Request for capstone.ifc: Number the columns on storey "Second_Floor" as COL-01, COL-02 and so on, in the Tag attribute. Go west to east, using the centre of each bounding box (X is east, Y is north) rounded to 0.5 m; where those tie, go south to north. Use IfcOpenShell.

First a look at what the model holds.

```python
import ifcopenshell
import ifcopenshell.util.element
import ifcopenshell.util.placement

model = ifcopenshell.open("capstone.ifc")
print(model.schema)
storey = next(s for s in model.by_type("IfcBuildingStorey") if s.Name == "Second_Floor")
columns = [e for e in ifcopenshell.util.element.get_decomposition(storey) if e.is_a("IfcColumn")]
for e in sorted(columns, key=lambda e: e.id()):
    origin = ifcopenshell.util.placement.get_local_placement(e.ObjectPlacement)[:3, 3]
    print(e.id(), e.Tag, e.Name, origin.round(2) + 0.0, sep=" | ")
```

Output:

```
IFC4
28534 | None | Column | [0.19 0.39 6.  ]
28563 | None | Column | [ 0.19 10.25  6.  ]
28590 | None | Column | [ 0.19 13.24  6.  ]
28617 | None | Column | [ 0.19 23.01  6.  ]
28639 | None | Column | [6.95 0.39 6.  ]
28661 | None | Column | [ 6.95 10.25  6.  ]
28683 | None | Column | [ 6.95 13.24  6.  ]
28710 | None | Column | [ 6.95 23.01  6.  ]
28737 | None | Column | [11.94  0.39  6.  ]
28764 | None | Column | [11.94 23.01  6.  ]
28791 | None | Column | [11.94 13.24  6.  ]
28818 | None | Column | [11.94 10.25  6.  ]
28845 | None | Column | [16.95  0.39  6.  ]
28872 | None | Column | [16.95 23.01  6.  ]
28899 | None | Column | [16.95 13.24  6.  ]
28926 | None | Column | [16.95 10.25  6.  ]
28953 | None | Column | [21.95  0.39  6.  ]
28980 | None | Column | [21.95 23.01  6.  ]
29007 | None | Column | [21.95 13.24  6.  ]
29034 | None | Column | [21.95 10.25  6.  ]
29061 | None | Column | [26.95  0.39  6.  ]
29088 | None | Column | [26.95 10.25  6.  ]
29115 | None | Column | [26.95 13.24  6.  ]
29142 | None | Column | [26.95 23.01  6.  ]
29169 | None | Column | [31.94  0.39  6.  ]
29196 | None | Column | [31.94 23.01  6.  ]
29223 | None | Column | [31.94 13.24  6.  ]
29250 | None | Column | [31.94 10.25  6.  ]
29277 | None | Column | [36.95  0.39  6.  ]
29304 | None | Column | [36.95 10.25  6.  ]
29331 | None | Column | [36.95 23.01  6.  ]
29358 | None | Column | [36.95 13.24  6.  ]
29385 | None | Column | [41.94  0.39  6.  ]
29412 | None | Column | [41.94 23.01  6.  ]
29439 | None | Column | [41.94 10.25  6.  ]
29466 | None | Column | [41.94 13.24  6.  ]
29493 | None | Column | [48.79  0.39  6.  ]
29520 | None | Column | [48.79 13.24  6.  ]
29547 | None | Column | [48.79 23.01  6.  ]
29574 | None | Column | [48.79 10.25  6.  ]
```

```python
import ifcopenshell
import ifcopenshell.geom
import ifcopenshell.util.element
import ifcopenshell.util.shape

model = ifcopenshell.open("capstone.ifc")
settings = ifcopenshell.geom.settings()
settings.set("use-world-coords", True)


def centre(element):
    shape = ifcopenshell.geom.create_shape(settings, element)
    return ifcopenshell.util.shape.get_bbox_centroid(shape.geometry)


storey = next(s for s in model.by_type("IfcBuildingStorey") if s.Name == "Second_Floor")
columns = [e for e in ifcopenshell.util.element.get_decomposition(storey) if e.is_a("IfcColumn")]

# Insertion points can sit at a corner or the storey origin, so sort by the geometry (in metres).
centres = {e: centre(e) for e in columns}
columns.sort(key=lambda e: (round(centres[e][0] / 0.5), centres[e][1]))

for i, e in enumerate(columns, start=1):
    number = f"COL-{i:02d}"
    e.Tag = number
    print(e.id(), number)

model.write("capstone_rev.ifc")
```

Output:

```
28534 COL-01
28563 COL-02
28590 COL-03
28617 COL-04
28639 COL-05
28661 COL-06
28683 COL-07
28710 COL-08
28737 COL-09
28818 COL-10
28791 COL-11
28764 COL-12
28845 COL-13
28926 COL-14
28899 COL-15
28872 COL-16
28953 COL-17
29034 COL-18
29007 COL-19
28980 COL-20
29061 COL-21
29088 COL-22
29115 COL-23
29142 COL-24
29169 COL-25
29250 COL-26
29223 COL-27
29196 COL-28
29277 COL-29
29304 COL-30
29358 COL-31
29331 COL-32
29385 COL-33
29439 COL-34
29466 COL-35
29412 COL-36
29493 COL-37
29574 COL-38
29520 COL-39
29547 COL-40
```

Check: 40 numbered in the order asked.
